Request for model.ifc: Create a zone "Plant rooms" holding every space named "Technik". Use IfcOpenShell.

First a look at what the model holds.

```python
import ifcopenshell

model = ifcopenshell.open("model.ifc")
print(model.schema)
seen = {}
for space in model.by_type("IfcSpace"):
    seen[space.LongName] = seen.get(space.LongName, 0) + 1
for name, count in sorted(seen.items(), key=str):
    print(count, "x", name)
print("zones:", [z.Name for z in model.by_type("IfcZone")][:20])
```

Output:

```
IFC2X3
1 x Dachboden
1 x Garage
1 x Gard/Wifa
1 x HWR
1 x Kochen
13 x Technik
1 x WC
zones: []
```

```python
import ifcopenshell
import ifcopenshell.api.group
import ifcopenshell.api.root

model = ifcopenshell.open("model.ifc")

names = {"Technik"}
spaces = [s for s in model.by_type("IfcSpace") if s.LongName in names]

zone = ifcopenshell.api.root.create_entity(model, ifc_class="IfcZone", name="Plant rooms")
ifcopenshell.api.group.assign_group(model, products=spaces, group=zone)
print(len(spaces), "spaces in", zone.Name)

model.write("model_rev.ifc")
```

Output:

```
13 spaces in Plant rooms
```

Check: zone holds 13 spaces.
